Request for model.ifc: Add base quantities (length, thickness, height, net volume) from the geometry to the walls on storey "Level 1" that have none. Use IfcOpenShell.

First a look at what the model holds.

```python
import ifcopenshell
import ifcopenshell.util.element
import ifcopenshell.util.unit

model = ifcopenshell.open("model.ifc")
print(model.schema)
for unit_type in ("LENGTHUNIT", "AREAUNIT", "VOLUMEUNIT"):
    print(unit_type, ifcopenshell.util.unit.calculate_unit_scale(model, unit_type))
storey = next(s for s in model.by_type("IfcBuildingStorey") if s.Name == "Level 1")
walls = [e for e in ifcopenshell.util.element.get_decomposition(storey) if e.is_a("IfcWall")]
for e in sorted(walls, key=lambda e: e.id()):
    print(e.id(), e.is_a(), e.Name, list(ifcopenshell.util.element.get_psets(e, qtos_only=True)), sep=" | ")
```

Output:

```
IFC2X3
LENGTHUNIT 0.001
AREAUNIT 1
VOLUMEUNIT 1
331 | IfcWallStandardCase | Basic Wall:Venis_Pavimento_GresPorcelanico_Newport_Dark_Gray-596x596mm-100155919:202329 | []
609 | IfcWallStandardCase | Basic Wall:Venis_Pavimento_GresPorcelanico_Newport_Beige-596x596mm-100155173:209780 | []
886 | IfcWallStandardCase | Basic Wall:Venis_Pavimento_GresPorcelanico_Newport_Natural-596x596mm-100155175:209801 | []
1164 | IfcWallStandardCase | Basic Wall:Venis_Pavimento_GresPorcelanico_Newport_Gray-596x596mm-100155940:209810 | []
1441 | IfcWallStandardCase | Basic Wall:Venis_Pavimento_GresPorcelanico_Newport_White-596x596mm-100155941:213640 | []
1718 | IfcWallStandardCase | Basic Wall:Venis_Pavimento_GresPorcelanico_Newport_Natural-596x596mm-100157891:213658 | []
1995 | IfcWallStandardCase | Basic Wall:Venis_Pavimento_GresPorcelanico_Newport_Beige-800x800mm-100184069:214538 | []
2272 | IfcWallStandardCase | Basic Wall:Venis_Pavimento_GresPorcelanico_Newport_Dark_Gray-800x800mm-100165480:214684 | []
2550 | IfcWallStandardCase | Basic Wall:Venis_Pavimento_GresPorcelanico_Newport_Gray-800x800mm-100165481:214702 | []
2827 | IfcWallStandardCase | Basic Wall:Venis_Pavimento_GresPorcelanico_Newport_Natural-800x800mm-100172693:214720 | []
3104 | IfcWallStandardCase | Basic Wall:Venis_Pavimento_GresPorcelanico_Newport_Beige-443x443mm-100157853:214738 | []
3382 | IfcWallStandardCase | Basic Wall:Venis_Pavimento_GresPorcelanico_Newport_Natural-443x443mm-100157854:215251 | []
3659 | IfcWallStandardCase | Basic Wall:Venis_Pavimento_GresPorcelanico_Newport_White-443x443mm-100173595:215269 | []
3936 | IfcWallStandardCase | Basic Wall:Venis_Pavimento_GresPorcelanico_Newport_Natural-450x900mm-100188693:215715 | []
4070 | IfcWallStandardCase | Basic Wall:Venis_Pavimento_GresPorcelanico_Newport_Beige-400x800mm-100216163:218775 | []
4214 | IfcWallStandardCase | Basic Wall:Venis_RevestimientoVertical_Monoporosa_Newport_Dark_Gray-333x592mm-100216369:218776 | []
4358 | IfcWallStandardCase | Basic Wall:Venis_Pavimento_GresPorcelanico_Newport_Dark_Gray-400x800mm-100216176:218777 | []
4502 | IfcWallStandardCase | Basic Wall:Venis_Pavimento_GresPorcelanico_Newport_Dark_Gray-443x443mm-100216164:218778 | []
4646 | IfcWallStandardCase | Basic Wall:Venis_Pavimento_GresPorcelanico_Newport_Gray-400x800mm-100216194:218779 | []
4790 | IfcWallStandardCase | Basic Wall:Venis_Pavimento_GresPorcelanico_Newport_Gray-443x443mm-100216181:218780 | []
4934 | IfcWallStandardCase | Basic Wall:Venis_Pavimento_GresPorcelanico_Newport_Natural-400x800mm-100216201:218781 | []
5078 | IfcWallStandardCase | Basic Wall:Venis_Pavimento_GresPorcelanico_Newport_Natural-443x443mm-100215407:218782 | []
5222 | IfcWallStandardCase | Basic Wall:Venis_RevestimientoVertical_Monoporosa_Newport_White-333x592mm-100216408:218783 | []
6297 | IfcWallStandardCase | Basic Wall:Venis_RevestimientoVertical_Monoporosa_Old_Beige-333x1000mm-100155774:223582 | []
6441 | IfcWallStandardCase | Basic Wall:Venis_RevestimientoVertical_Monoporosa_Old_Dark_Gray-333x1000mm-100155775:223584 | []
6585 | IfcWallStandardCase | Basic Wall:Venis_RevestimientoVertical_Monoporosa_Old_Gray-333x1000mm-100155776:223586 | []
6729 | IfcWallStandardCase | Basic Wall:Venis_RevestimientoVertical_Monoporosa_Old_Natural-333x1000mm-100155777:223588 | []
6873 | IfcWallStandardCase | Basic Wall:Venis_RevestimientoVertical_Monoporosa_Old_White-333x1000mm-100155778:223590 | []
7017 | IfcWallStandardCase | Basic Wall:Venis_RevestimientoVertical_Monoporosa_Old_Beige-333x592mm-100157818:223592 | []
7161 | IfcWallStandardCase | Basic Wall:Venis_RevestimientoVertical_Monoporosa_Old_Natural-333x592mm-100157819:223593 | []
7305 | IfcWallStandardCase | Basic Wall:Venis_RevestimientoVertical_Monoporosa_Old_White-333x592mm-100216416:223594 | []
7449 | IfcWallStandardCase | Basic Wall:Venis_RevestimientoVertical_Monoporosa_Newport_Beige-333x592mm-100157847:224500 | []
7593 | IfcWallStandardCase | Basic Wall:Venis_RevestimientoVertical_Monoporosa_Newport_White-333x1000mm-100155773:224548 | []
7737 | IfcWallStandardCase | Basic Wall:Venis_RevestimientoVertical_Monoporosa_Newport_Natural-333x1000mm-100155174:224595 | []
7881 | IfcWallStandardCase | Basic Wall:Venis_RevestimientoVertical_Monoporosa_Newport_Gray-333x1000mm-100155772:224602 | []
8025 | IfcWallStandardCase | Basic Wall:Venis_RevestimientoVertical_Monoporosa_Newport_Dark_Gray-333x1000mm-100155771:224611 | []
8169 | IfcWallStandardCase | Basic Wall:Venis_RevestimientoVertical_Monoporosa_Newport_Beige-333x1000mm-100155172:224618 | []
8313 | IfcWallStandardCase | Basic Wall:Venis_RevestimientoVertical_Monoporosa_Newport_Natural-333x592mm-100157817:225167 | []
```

```python
import ifcopenshell
import ifcopenshell.api.pset
import ifcopenshell.geom
import ifcopenshell.util.element
import ifcopenshell.util.shape
import ifcopenshell.util.unit

model = ifcopenshell.open("model.ifc")
unit_scale = ifcopenshell.util.unit.calculate_unit_scale(model)
volume_scale = ifcopenshell.util.unit.calculate_unit_scale(model, "VOLUMEUNIT")
settings = ifcopenshell.geom.settings()

storey = next(s for s in model.by_type("IfcBuildingStorey") if s.Name == "Level 1")
walls = [e for e in ifcopenshell.util.element.get_decomposition(storey) if e.is_a("IfcWall")]

for e in sorted(walls, key=lambda e: e.id()):
    if ifcopenshell.util.element.get_psets(e, qtos_only=True, should_inherit=False):
        continue
    # Geometry comes back in metres, in the element's own axes.
    shape = ifcopenshell.geom.create_shape(settings, e)
    values = {
        "Length": ifcopenshell.util.shape.get_x(shape.geometry) / unit_scale,
        "Width": ifcopenshell.util.shape.get_y(shape.geometry) / unit_scale,
        "Height": ifcopenshell.util.shape.get_z(shape.geometry) / unit_scale,
        "NetVolume": ifcopenshell.util.shape.get_volume(shape.geometry) / volume_scale,
    }
    qto = ifcopenshell.api.pset.add_qto(model, product=e, name="BaseQuantities")
    ifcopenshell.api.pset.edit_qto(model, qto=qto, properties=values)
    print(e.id(), {k: round(v, 3) for k, v in values.items()})

model.write("model-out.ifc")
```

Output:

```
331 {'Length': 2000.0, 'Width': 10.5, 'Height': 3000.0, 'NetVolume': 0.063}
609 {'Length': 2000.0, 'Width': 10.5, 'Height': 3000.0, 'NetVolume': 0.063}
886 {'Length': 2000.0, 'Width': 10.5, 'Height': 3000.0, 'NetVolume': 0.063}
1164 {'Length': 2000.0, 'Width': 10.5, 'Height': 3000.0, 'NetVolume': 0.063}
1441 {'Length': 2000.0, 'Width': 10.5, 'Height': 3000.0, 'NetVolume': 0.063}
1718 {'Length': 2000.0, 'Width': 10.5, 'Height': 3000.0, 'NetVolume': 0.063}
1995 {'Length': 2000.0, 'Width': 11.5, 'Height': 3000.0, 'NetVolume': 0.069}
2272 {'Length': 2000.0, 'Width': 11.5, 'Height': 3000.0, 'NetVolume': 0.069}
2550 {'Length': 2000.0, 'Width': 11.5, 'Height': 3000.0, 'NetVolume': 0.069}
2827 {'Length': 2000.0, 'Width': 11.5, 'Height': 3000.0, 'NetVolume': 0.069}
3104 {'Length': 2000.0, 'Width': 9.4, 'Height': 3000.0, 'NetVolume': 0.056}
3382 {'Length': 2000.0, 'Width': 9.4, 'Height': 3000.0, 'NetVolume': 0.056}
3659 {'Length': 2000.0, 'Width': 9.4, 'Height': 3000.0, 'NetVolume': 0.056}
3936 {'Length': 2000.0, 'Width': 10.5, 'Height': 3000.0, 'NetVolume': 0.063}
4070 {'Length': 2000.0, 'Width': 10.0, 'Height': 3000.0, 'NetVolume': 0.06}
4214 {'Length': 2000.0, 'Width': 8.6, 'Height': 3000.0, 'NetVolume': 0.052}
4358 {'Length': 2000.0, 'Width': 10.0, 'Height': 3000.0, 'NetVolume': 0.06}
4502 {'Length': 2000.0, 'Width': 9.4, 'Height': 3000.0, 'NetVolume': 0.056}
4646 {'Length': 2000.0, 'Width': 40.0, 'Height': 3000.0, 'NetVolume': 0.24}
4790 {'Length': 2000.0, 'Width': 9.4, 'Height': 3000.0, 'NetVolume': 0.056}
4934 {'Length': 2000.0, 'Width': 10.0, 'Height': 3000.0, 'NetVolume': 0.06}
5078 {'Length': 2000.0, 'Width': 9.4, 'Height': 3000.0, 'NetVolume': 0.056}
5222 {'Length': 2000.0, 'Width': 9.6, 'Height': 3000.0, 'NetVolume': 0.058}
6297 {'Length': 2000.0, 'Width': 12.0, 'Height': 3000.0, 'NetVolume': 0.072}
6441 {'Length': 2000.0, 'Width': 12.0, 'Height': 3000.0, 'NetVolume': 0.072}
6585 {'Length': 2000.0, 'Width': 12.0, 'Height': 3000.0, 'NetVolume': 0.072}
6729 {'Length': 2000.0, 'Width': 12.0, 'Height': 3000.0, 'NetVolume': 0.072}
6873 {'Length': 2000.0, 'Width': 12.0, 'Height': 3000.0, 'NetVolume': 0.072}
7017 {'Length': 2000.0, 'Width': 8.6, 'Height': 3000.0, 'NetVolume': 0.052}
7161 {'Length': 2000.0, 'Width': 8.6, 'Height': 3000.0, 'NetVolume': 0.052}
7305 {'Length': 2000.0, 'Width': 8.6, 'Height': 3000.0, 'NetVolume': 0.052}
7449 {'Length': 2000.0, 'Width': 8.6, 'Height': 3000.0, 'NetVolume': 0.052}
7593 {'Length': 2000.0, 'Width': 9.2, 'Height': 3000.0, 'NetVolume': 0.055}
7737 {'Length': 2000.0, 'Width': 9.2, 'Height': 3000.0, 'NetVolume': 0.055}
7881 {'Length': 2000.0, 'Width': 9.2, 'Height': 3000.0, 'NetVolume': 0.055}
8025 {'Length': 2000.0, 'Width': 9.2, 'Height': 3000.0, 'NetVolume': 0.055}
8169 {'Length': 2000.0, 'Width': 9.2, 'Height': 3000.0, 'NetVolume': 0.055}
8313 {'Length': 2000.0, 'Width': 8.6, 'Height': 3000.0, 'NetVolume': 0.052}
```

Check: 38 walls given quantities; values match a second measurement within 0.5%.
